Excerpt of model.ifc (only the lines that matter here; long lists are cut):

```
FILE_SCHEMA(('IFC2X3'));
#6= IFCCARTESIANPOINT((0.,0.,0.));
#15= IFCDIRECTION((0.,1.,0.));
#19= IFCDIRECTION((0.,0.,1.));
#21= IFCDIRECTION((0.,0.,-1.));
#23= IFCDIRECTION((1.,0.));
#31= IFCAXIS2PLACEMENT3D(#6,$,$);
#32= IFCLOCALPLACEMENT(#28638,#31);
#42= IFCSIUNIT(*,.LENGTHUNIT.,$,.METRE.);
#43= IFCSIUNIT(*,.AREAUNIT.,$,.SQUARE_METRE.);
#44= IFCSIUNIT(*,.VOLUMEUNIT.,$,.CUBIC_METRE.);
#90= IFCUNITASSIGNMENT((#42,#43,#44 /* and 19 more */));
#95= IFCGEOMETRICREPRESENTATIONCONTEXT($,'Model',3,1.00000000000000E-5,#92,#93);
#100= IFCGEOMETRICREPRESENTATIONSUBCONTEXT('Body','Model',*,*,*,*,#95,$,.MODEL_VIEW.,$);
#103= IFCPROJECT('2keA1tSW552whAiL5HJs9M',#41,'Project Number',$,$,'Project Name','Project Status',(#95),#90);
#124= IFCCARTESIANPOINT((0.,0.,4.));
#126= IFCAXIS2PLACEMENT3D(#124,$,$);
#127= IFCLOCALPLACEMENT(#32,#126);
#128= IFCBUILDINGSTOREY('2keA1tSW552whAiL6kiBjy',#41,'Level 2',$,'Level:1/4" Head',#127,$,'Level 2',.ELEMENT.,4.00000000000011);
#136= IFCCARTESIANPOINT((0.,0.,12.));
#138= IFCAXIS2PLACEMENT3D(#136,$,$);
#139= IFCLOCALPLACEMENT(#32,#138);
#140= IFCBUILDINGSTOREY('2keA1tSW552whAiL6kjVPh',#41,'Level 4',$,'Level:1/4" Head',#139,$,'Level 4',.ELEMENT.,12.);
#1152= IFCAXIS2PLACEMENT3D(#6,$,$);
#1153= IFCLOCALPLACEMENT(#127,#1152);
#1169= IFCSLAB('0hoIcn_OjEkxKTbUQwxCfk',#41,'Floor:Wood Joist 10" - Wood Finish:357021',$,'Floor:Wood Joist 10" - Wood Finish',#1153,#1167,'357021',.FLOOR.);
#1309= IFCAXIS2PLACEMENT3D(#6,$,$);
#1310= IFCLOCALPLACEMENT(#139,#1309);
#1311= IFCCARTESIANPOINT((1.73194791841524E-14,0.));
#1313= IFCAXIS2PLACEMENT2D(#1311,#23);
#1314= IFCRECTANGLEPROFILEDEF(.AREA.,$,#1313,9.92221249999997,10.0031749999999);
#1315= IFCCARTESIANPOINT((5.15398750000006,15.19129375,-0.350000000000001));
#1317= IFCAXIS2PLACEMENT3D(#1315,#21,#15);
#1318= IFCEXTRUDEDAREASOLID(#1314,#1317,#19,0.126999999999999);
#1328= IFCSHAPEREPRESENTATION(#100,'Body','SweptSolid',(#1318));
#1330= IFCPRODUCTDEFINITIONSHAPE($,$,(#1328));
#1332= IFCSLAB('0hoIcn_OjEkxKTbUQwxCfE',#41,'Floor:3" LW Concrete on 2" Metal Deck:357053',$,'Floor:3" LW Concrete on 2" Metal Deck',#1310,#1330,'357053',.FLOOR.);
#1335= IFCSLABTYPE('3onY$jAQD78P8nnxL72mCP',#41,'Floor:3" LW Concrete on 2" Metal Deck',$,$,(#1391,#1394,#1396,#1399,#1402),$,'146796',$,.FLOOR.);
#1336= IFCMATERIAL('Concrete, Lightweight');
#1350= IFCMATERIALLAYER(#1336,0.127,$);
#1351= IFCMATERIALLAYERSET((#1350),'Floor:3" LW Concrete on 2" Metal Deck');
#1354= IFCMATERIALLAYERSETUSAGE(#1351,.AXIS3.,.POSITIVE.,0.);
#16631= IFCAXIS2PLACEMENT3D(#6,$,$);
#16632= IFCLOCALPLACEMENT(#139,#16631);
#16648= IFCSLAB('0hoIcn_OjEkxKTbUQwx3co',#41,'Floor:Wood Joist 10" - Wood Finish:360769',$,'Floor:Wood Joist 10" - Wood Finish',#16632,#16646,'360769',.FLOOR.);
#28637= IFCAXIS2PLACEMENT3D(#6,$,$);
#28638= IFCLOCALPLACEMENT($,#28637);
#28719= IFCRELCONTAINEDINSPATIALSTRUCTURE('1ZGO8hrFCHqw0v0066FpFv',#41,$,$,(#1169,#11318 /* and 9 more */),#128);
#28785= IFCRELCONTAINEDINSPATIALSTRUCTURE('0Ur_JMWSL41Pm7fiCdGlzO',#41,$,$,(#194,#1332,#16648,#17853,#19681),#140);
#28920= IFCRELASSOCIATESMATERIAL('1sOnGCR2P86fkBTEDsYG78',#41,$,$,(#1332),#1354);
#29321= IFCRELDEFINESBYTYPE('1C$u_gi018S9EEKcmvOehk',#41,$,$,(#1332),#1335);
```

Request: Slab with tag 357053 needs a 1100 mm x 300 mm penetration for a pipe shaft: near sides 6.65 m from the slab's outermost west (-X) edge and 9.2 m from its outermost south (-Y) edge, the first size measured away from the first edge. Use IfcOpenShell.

```python
import numpy as np
import ifcopenshell
import ifcopenshell.api.feature
import ifcopenshell.api.geometry
import ifcopenshell.api.root
import ifcopenshell.geom
import ifcopenshell.util.placement
import ifcopenshell.util.representation
import ifcopenshell.util.shape
import ifcopenshell.util.unit

model = ifcopenshell.open("model.ifc")
unit_scale = ifcopenshell.util.unit.calculate_unit_scale(model)
settings = ifcopenshell.geom.settings()


def volume(element):
    """Net volume in cubic metres, openings subtracted."""
    shape = ifcopenshell.geom.create_shape(settings, element)
    return ifcopenshell.util.shape.get_volume(shape.geometry)


slab = model.by_guid("0hoIcn_OjEkxKTbUQwxCfE")
before = volume(slab)

# Extent in the slab's own axes, in metres. The edges named are its -X and -Y sides.
slab_shape = ifcopenshell.geom.create_shape(settings, slab)
vertices = ifcopenshell.util.shape.get_vertices(slab_shape.geometry)
x_min, y_min, bottom = vertices.min(axis=0)
top = vertices[:, 2].max()

opening = ifcopenshell.api.root.create_entity(model, ifc_class="IfcOpeningElement", name="Pipe shaft opening")
context = ifcopenshell.util.representation.get_context(model, "Model", "Body", "MODEL_VIEW")
width, depth = 1.1, 0.3
outline = [(0.0, 0.0), (width, 0.0), (width, depth), (0.0, depth), (0.0, 0.0)]
# Overshoot both faces by 50 mm so the cut is clean.
shape = ifcopenshell.api.geometry.add_slab_representation(
    model, context=context, depth=top - bottom + 0.1, polyline=outline
)
ifcopenshell.api.geometry.assign_representation(model, product=opening, representation=shape)

matrix = ifcopenshell.util.placement.get_local_placement(slab.ObjectPlacement)
matrix[:, 3] = matrix @ np.append(np.array([x_min + 6.65, y_min + 9.2, bottom - 0.05]) / unit_scale, 1.0)
ifcopenshell.api.geometry.edit_object_placement(model, product=opening, matrix=matrix, is_si=False)
ifcopenshell.api.feature.add_feature(model, feature=opening, element=slab)

after = volume(slab)

print(f"slab volume {before:.3f} -> {after:.3f} m3")

model.write("model_rev.ifc")
```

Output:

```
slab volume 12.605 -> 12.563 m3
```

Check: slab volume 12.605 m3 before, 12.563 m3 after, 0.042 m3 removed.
